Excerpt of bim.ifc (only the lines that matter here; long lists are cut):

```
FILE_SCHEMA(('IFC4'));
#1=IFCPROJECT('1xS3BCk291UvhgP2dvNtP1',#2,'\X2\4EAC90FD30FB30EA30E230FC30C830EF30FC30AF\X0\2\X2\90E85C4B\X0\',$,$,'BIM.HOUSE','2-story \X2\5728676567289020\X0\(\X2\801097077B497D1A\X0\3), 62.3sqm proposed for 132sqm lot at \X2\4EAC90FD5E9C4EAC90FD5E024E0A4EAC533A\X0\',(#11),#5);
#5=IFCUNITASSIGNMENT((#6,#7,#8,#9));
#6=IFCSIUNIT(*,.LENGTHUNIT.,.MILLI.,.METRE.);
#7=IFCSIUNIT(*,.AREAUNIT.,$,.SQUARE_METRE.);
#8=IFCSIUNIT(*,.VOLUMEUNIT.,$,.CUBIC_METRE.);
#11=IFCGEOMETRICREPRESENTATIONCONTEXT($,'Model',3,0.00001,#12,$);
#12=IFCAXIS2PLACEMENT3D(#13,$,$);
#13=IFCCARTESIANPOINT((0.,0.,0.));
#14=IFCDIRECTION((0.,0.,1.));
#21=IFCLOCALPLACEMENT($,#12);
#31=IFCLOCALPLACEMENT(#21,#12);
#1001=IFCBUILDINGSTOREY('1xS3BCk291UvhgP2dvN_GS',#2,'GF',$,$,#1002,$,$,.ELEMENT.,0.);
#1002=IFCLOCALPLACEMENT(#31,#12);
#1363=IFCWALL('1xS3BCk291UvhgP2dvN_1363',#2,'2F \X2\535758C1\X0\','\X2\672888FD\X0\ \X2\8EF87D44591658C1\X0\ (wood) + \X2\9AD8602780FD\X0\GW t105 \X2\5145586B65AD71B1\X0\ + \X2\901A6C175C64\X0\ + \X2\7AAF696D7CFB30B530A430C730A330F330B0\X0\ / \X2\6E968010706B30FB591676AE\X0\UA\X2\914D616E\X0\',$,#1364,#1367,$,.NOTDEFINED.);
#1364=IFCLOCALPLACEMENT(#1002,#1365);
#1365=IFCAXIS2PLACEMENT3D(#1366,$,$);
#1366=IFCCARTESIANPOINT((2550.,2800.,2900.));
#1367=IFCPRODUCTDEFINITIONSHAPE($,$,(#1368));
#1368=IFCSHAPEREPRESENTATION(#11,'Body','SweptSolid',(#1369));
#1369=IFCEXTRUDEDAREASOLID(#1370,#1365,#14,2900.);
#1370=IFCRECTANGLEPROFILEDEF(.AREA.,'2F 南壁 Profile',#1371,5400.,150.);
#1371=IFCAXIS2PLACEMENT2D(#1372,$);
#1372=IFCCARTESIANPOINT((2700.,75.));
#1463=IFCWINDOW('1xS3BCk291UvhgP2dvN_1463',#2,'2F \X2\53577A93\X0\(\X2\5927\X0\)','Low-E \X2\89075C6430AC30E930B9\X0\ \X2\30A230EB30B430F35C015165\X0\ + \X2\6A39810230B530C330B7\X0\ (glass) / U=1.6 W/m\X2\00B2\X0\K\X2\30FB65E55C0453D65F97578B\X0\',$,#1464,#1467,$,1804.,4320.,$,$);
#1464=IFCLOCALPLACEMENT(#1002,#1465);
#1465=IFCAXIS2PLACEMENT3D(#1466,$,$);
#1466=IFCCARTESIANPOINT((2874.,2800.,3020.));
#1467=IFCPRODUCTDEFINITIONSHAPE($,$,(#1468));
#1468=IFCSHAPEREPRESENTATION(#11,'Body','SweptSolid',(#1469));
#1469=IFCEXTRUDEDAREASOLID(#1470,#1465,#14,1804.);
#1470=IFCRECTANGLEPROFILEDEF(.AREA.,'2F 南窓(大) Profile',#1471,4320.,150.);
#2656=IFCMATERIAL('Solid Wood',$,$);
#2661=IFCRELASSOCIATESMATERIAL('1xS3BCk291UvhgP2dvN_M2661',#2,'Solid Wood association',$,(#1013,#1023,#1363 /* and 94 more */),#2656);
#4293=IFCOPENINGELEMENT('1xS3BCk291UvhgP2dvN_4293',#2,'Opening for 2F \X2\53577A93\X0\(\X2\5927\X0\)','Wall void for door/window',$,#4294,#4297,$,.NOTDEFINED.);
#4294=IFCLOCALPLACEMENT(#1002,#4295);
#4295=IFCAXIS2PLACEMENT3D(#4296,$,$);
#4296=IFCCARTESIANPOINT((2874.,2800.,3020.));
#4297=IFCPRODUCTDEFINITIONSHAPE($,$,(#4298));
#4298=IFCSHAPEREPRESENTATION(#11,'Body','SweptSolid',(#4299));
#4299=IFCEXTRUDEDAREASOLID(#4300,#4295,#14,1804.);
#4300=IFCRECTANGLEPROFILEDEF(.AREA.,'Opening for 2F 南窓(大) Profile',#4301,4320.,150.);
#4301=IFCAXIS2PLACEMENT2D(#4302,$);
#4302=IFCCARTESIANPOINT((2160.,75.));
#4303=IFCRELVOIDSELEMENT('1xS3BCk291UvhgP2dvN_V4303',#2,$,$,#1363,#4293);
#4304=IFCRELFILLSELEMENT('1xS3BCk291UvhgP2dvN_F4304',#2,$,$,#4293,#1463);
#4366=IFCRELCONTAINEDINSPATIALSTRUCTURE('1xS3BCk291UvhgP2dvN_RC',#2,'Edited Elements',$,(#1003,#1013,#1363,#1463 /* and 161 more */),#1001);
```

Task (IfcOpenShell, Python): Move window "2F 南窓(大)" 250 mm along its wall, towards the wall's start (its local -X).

```python
import ifcopenshell
import ifcopenshell.api.geometry
import ifcopenshell.util.placement
import ifcopenshell.util.unit

model = ifcopenshell.open("bim.ifc")
unit_scale = ifcopenshell.util.unit.calculate_unit_scale(model)

window = model.by_id(1463)
opening = window.FillsVoids[0].RelatingOpeningElement
wall = opening.VoidsElements[0].RelatingBuildingElement

wall_matrix = ifcopenshell.util.placement.get_local_placement(wall.ObjectPlacement)
shift = wall_matrix[:3, 0] * -0.25 / unit_scale
before = ifcopenshell.util.placement.get_local_placement(window.ObjectPlacement)[:3, 3].copy()

# The window is not placed relative to its opening, so move both.
for product in (opening, window):
    matrix = ifcopenshell.util.placement.get_local_placement(product.ObjectPlacement)
    matrix[:3, 3] += shift
    ifcopenshell.api.geometry.edit_object_placement(model, product=product, matrix=matrix, is_si=False)

after = ifcopenshell.util.placement.get_local_placement(window.ObjectPlacement)[:3, 3]
print("window moved by", (after - before).round(3) + 0.0)

model.write("bim_edited.ifc")
```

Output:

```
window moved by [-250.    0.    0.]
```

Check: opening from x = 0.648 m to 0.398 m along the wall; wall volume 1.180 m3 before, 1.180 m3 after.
